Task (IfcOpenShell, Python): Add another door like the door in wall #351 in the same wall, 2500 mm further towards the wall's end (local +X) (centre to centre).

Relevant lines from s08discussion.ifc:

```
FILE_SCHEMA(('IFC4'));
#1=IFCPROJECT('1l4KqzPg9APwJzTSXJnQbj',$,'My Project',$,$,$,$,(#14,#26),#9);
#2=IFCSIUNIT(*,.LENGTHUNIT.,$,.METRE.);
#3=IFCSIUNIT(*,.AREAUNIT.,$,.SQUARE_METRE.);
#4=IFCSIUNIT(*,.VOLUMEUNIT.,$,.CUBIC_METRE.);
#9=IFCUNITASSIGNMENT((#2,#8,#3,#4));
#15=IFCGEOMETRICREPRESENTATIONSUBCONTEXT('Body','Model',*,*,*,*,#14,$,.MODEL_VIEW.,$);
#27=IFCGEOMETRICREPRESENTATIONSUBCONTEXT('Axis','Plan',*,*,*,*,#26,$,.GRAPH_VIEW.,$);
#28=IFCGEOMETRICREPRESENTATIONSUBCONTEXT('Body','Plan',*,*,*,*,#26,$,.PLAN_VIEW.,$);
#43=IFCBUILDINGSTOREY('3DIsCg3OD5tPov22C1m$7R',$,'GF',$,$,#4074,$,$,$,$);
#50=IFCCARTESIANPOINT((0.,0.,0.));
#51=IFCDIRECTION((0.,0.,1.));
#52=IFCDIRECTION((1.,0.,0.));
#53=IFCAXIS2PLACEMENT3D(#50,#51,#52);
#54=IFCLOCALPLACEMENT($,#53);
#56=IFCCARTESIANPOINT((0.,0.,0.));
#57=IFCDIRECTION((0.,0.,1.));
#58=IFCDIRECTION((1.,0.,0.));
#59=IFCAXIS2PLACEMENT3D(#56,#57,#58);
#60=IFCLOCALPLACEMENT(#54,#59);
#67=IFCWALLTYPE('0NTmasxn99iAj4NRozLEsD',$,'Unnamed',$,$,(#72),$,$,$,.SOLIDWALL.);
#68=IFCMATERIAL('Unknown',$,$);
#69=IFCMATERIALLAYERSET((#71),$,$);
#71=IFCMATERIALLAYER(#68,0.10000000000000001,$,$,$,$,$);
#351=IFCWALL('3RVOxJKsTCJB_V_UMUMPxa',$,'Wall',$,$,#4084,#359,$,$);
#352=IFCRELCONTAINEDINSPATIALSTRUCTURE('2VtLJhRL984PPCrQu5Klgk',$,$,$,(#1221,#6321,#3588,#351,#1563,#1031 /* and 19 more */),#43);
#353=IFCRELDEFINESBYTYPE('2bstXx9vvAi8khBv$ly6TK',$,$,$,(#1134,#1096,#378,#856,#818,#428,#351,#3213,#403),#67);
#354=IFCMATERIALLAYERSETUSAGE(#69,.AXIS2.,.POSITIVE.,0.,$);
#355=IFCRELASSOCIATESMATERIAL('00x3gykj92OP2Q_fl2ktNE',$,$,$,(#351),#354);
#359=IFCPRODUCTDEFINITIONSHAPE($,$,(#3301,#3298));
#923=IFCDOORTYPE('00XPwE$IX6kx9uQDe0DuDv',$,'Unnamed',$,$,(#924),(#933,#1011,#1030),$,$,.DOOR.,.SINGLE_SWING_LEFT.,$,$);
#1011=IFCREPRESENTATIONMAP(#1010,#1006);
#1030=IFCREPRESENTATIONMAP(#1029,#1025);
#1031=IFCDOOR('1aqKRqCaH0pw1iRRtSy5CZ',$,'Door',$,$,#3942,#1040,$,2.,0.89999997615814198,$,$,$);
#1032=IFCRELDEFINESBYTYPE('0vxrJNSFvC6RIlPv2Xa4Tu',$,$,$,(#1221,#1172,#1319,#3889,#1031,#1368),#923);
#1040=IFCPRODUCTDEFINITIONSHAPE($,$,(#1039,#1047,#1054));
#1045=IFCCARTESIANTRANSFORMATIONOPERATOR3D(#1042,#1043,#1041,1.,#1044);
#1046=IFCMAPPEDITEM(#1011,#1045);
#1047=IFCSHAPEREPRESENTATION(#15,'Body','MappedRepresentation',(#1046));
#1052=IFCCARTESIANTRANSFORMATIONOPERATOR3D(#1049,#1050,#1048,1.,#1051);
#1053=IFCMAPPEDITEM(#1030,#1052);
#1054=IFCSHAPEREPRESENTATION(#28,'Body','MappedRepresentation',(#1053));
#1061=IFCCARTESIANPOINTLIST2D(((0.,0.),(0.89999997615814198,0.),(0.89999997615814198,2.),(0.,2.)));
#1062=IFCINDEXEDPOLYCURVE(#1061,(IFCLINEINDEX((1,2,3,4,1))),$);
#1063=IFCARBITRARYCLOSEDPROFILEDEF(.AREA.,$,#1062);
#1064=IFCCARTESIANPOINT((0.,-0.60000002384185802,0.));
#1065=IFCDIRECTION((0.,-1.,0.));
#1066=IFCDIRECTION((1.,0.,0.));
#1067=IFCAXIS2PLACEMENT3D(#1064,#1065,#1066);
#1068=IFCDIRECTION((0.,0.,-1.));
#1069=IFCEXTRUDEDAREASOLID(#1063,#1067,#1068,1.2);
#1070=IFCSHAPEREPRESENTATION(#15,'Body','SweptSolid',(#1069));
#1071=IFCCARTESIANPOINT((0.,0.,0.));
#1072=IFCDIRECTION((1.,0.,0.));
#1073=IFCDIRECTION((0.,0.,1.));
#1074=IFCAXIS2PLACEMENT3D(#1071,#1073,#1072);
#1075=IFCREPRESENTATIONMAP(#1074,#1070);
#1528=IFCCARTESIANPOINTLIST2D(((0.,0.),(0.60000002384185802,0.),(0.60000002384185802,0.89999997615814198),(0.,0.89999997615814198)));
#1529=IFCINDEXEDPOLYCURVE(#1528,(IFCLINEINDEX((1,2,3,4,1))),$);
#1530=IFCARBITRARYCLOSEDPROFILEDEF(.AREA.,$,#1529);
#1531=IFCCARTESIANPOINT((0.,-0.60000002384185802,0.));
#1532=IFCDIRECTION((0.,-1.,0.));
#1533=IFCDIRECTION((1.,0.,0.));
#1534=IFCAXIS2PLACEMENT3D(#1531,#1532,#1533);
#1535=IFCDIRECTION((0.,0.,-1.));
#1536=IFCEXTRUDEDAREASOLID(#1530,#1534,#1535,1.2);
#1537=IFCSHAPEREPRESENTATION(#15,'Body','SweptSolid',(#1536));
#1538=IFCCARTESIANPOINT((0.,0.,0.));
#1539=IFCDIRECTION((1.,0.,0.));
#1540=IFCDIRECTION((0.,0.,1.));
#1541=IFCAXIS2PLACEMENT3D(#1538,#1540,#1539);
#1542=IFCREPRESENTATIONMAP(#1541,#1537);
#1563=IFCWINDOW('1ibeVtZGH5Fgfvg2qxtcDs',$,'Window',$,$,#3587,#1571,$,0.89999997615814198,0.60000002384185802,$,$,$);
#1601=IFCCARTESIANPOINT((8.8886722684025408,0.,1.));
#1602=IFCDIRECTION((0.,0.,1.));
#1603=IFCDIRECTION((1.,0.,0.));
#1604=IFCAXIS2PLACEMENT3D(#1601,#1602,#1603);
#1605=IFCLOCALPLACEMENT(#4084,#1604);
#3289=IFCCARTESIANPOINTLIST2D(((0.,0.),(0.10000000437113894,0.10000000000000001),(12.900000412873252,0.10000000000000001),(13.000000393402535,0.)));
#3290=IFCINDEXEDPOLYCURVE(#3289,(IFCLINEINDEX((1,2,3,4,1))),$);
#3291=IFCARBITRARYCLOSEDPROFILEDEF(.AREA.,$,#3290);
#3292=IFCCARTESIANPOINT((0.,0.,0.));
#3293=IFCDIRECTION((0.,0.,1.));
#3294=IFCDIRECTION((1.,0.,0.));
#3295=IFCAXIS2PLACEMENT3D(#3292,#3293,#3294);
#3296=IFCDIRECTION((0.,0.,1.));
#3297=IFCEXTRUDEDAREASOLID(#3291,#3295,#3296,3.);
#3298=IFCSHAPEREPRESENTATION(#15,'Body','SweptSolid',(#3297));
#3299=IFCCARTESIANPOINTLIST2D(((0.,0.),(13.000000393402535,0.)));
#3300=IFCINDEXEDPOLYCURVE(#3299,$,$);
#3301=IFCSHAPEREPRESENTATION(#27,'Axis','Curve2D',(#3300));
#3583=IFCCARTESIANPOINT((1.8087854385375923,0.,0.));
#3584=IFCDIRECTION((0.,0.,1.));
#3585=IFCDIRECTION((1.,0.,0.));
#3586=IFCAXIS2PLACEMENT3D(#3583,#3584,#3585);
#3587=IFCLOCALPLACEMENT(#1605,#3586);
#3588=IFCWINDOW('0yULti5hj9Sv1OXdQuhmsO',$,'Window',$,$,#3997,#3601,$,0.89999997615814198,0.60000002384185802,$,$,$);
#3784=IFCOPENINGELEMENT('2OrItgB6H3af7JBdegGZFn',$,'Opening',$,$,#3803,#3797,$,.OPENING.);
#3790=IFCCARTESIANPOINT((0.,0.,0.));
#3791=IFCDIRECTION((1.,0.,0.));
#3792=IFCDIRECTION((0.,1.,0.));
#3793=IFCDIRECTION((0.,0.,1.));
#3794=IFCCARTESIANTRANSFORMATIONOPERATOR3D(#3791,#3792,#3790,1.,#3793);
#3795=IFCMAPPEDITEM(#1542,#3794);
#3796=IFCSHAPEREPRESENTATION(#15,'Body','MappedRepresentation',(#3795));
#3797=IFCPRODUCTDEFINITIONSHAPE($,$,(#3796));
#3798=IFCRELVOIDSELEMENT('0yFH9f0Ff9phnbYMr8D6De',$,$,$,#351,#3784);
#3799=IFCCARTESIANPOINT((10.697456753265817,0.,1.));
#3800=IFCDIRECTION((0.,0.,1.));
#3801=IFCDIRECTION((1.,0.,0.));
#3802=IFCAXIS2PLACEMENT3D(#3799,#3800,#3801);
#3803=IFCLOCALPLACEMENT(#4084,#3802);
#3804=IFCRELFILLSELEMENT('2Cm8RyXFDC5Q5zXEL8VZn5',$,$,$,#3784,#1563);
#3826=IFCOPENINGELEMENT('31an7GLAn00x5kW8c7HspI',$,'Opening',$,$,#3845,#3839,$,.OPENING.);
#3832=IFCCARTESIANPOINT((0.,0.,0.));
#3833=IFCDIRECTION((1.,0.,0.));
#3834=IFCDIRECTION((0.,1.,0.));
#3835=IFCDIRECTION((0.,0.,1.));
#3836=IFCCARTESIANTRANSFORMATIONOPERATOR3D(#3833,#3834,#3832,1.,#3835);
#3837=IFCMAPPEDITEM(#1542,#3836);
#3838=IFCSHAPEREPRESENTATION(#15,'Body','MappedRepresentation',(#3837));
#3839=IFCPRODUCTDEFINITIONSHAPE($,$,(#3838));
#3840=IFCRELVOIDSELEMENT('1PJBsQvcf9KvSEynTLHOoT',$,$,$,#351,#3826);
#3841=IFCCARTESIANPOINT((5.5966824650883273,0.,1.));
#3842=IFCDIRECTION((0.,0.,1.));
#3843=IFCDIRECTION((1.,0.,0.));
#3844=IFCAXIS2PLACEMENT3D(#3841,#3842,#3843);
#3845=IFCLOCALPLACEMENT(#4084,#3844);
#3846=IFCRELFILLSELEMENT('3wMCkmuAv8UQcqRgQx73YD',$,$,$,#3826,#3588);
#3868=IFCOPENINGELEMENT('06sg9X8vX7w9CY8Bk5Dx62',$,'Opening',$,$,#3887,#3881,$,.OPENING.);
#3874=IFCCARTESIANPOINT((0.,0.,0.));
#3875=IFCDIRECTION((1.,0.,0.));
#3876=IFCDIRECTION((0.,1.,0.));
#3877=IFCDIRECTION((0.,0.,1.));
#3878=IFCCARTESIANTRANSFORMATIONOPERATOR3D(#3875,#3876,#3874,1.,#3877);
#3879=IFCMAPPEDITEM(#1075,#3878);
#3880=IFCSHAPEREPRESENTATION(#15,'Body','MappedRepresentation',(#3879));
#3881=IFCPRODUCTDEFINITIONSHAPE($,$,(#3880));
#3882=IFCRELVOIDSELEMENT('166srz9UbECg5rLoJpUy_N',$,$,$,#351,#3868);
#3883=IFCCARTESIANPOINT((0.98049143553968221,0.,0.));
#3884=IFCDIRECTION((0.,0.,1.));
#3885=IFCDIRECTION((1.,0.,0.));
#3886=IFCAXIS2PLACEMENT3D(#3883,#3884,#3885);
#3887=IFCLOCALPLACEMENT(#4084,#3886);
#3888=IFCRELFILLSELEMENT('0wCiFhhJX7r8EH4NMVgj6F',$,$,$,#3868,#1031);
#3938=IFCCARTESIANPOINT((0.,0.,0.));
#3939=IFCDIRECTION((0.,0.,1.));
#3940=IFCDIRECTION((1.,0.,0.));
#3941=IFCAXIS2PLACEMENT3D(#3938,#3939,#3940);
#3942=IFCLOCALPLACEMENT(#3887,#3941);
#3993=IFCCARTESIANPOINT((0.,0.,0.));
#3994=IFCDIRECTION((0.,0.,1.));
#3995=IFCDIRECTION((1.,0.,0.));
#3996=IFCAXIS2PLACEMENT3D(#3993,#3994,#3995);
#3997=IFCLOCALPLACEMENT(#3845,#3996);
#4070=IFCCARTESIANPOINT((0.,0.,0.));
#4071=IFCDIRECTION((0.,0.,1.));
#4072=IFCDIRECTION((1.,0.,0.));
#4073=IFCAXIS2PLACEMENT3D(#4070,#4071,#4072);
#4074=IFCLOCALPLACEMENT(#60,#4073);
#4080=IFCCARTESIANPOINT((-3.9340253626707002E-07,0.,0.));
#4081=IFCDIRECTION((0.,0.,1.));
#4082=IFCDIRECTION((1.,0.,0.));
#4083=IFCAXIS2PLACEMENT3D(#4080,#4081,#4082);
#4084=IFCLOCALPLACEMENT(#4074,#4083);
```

```python
import ifcopenshell
import ifcopenshell.api.feature
import ifcopenshell.api.geometry
import ifcopenshell.api.root
import ifcopenshell.geom
import ifcopenshell.util.element
import ifcopenshell.util.placement
import ifcopenshell.util.shape

model = ifcopenshell.open("s08discussion.ifc")
settings = ifcopenshell.geom.settings()


def volume(element):
    """Net volume in cubic metres, openings subtracted."""
    shape = ifcopenshell.geom.create_shape(settings, element)
    return ifcopenshell.util.shape.get_volume(shape.geometry)


door = model.by_guid("1aqKRqCaH0pw1iRRtSy5CZ")
opening = door.FillsVoids[0].RelatingOpeningElement
wall = opening.VoidsElements[0].RelatingBuildingElement
before = volume(wall)
shift = ifcopenshell.util.placement.get_local_placement(wall.ObjectPlacement)[:3, 0] * 2.5

# copy_class copies the void relationship, type, container and properties, but no geometry.
new_opening = ifcopenshell.api.root.copy_class(model, product=opening)
new_opening.Representation = ifcopenshell.util.element.copy_deep(
    model, opening.Representation, exclude=["IfcGeometricRepresentationContext", "IfcRepresentationMap"]
)
new_door = ifcopenshell.api.root.copy_class(model, product=door)
new_door.Representation = ifcopenshell.util.element.copy_deep(
    model, door.Representation, exclude=["IfcGeometricRepresentationContext", "IfcRepresentationMap"]
)
ifcopenshell.api.feature.add_filling(model, opening=new_opening, element=new_door)

for old, new in ((opening, new_opening), (door, new_door)):
    matrix = ifcopenshell.util.placement.get_local_placement(old.ObjectPlacement)
    matrix[:3, 3] += shift
    ifcopenshell.api.geometry.edit_object_placement(model, product=new, matrix=matrix, is_si=False)

after = volume(wall)

print(f"wall volume {before:.3f} -> {after:.3f} m3")

model.write("s08discussion-out.ifc")
```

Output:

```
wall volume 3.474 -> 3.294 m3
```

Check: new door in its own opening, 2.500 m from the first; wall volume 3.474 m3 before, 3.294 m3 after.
